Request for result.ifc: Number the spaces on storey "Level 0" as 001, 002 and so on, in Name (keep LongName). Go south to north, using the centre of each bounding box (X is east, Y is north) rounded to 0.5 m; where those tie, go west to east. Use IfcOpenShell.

First a look at what the model holds.

```python
import ifcopenshell
import ifcopenshell.util.element
import ifcopenshell.util.placement

model = ifcopenshell.open("result.ifc")
print(model.schema)
storey = next(s for s in model.by_type("IfcBuildingStorey") if s.Name == "Level 0")
spaces = [e for e in ifcopenshell.util.element.get_decomposition(storey) if e.is_a("IfcSpace")]
for e in sorted(spaces, key=lambda e: e.id()):
    origin = ifcopenshell.util.placement.get_local_placement(e.ObjectPlacement)[:3, 3]
    print(e.id(), e.Name, e.LongName, origin.round(2) + 0.0, sep=" | ")
```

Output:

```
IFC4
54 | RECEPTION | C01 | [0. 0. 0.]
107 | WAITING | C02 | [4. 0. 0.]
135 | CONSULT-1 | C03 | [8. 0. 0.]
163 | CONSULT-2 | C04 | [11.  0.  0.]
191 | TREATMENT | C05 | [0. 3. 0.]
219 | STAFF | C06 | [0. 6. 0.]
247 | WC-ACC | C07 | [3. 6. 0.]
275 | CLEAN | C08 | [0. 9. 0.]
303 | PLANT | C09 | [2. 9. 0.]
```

```python
import ifcopenshell
import ifcopenshell.geom
import ifcopenshell.util.element
import ifcopenshell.util.shape

model = ifcopenshell.open("result.ifc")
settings = ifcopenshell.geom.settings()
settings.set("use-world-coords", True)


def centre(element):
    shape = ifcopenshell.geom.create_shape(settings, element)
    return ifcopenshell.util.shape.get_bbox_centroid(shape.geometry)


storey = next(s for s in model.by_type("IfcBuildingStorey") if s.Name == "Level 0")
spaces = [e for e in ifcopenshell.util.element.get_decomposition(storey) if e.is_a("IfcSpace")]

# Insertion points can sit at a corner or the storey origin, so sort by the geometry (in metres).
centres = {e: centre(e) for e in spaces}
spaces.sort(key=lambda e: (round(centres[e][1] / 0.5), centres[e][0]))

for i, e in enumerate(spaces, start=1):
    number = f"0{i:02d}"
    e.Name = number
    print(e.id(), number)

model.write("result-out.ifc")
```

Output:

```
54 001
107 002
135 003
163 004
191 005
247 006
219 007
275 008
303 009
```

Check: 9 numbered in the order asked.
